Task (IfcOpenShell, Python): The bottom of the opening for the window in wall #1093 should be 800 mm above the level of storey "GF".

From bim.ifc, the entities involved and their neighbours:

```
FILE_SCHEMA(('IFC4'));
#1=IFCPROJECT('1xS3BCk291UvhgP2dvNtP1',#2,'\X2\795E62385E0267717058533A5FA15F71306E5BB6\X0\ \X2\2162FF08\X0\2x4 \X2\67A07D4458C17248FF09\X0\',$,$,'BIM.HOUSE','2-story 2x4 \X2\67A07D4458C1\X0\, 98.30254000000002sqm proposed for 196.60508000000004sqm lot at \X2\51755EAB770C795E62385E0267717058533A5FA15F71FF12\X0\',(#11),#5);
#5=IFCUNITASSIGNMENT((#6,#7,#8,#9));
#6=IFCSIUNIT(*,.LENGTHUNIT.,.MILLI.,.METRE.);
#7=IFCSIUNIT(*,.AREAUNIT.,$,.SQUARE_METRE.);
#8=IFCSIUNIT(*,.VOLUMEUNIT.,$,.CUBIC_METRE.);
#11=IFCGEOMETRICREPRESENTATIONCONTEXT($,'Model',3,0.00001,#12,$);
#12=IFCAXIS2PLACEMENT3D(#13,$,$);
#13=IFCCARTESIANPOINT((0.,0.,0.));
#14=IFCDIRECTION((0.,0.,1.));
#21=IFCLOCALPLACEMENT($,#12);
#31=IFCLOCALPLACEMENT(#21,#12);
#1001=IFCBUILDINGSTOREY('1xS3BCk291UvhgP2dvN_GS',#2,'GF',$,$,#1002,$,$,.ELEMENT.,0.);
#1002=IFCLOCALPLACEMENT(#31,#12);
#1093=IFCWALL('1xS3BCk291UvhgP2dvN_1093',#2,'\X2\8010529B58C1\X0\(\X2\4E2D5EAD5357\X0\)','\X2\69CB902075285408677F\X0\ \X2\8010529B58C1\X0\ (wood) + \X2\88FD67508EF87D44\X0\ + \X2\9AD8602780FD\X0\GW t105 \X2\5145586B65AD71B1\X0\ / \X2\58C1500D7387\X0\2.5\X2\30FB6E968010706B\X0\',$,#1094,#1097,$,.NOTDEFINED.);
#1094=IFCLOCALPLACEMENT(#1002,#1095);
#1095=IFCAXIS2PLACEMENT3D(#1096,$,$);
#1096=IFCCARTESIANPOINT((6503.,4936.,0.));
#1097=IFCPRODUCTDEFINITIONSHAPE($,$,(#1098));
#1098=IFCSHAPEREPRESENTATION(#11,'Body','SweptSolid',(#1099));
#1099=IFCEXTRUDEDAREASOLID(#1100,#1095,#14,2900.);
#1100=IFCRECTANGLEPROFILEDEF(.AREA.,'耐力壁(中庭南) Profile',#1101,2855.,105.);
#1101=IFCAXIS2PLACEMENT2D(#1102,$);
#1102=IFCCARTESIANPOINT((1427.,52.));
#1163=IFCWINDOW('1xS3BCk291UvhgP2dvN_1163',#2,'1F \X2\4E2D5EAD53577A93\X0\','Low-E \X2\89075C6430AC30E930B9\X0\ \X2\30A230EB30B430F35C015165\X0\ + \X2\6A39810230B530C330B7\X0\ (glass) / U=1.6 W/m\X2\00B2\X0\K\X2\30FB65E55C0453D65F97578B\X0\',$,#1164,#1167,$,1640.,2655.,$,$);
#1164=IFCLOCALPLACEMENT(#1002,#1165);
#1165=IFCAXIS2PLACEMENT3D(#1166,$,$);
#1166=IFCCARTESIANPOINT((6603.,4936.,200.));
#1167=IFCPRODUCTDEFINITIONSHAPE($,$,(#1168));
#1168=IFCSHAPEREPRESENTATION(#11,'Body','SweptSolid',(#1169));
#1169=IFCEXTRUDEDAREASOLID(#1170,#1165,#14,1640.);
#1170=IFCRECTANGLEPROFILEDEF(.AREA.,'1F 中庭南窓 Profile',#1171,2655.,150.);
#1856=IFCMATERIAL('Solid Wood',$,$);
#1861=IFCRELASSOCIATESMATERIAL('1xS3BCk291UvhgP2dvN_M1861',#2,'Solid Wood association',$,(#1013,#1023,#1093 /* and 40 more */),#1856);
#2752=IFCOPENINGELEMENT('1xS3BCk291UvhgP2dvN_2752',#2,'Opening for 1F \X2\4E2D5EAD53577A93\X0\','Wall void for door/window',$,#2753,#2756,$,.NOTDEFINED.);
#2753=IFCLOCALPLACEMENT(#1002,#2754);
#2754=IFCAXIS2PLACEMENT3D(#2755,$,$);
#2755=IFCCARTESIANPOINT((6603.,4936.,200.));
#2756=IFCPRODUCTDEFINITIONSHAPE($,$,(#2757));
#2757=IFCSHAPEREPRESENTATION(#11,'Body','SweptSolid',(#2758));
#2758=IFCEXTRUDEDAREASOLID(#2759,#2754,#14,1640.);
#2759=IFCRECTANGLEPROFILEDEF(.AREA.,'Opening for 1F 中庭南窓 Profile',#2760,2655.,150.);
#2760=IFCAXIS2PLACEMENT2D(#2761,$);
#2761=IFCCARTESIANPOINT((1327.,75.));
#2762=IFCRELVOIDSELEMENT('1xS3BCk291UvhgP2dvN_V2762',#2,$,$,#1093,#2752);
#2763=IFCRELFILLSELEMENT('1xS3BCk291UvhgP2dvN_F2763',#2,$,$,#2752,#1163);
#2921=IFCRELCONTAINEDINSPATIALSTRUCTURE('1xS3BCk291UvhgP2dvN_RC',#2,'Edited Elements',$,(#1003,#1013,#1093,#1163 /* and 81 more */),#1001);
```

```python
import numpy as np
import ifcopenshell
import ifcopenshell.api.geometry
import ifcopenshell.geom
import ifcopenshell.util.element
import ifcopenshell.util.placement
import ifcopenshell.util.shape
import ifcopenshell.util.unit

model = ifcopenshell.open("bim.ifc")
unit_scale = ifcopenshell.util.unit.calculate_unit_scale(model)

window = model.by_guid("1xS3BCk291UvhgP2dvN_1163")
opening = window.FillsVoids[0].RelatingOpeningElement
storey = ifcopenshell.util.element.get_container(window, ifc_class="IfcBuildingStorey")
level = ifcopenshell.util.placement.get_local_placement(storey.ObjectPlacement)[2, 3]

# The opening's origin need not be at the sill, so measure its lowest point.
shape = ifcopenshell.geom.create_shape(ifcopenshell.geom.settings(), opening)
bottom = ifcopenshell.util.shape.get_shape_bottom_elevation(shape, shape.geometry) / unit_scale
dz = level + 0.8 / unit_scale - bottom

shift = np.array([0.0, 0.0, dz])
# The window is not placed relative to its opening, so move both.
for product in (opening, window):
    matrix = ifcopenshell.util.placement.get_local_placement(product.ObjectPlacement)
    matrix[:3, 3] += shift
    ifcopenshell.api.geometry.edit_object_placement(model, product=product, matrix=matrix, is_si=False)

print(f"moved by {dz * unit_scale:+.3f} m")

model.write("bim_edited.ifc")
```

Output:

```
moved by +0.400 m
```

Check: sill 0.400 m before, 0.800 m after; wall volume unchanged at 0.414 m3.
